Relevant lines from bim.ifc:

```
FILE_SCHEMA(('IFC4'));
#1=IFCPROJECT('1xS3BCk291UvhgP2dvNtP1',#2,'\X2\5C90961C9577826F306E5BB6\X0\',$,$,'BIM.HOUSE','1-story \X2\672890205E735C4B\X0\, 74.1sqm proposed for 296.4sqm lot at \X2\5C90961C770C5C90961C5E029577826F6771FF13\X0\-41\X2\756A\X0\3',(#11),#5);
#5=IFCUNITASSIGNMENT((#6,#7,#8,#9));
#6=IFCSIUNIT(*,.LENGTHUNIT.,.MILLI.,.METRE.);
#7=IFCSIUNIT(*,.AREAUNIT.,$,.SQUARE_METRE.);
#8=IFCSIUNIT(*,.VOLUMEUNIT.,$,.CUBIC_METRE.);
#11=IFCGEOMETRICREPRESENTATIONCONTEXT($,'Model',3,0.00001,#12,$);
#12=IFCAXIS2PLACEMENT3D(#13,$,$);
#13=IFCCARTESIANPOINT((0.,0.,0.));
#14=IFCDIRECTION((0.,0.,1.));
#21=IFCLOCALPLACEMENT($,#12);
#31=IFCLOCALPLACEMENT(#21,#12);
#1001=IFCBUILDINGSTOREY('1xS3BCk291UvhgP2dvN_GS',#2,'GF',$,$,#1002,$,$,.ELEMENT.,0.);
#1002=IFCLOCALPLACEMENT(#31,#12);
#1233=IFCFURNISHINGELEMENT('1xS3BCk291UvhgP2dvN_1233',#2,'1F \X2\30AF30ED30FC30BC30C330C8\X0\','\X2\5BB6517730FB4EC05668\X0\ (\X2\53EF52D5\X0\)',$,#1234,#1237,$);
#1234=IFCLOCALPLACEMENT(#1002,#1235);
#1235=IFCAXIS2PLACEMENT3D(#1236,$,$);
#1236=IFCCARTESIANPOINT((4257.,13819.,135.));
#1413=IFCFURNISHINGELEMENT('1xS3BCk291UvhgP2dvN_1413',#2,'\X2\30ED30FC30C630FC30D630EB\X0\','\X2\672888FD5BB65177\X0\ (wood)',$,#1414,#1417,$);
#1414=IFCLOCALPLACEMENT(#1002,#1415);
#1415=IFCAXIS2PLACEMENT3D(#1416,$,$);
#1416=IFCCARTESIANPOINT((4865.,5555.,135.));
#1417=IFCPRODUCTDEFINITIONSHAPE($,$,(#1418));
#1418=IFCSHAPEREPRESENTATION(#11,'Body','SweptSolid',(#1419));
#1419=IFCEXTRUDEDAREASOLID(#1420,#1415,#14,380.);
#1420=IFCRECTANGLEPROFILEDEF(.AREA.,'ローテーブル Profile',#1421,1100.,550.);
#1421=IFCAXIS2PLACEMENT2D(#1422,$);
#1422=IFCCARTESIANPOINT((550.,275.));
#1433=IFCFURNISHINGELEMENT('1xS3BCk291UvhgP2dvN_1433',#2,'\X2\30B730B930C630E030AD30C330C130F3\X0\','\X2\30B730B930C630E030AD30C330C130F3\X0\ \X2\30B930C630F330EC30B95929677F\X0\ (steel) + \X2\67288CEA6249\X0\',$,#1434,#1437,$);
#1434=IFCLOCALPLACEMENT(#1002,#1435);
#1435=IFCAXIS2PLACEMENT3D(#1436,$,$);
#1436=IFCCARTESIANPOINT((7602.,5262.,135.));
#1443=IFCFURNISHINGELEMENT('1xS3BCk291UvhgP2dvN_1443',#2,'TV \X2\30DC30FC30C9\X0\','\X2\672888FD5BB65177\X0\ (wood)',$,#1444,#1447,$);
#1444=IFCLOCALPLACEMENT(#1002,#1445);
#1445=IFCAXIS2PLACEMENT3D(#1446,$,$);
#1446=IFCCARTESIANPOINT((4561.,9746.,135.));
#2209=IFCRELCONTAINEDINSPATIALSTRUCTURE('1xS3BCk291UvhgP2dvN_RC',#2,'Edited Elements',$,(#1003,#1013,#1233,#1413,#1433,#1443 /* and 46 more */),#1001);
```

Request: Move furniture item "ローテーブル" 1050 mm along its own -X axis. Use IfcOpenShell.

```python
import ifcopenshell
import ifcopenshell.api.geometry
import ifcopenshell.util.placement
import ifcopenshell.util.unit

model = ifcopenshell.open("bim.ifc")
unit_scale = ifcopenshell.util.unit.calculate_unit_scale(model)

item = model.by_guid("1xS3BCk291UvhgP2dvN_1413")
matrix = ifcopenshell.util.placement.get_local_placement(item.ObjectPlacement)
matrix[:3, 3] -= matrix[:3, 0] * 1.05 / unit_scale
ifcopenshell.api.geometry.edit_object_placement(model, product=item, matrix=matrix, is_si=False)

print(ifcopenshell.util.placement.get_local_placement(item.ObjectPlacement).round(3) + 0.0)

model.write("bim-out.ifc")
```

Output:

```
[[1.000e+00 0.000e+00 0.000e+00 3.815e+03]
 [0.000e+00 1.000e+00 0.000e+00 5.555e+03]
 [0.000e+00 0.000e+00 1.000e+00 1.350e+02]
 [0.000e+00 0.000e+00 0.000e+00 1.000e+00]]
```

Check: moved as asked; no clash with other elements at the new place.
